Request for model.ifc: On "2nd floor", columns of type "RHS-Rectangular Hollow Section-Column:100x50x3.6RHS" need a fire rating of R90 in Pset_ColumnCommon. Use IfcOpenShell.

First a look at what the model holds.

```python
import ifcopenshell
import ifcopenshell.util.element

model = ifcopenshell.open("model.ifc")
print(model.schema)
storey = next(s for s in model.by_type("IfcBuildingStorey") if s.Name == "2nd floor")
columns = [e for e in ifcopenshell.util.element.get_decomposition(storey) if e.is_a("IfcColumn")]
seen = {}
for e in columns:
    element_type = ifcopenshell.util.element.get_type(e)
    key = (element_type.Name if element_type != e and element_type else None, ifcopenshell.util.element.get_pset(e, "Pset_ColumnCommon", "FireRating"))
    seen[key] = seen.get(key, 0) + 1
for (name, value), count in sorted(seen.items(), key=str):
    print(count, "x", name, "|", value)
```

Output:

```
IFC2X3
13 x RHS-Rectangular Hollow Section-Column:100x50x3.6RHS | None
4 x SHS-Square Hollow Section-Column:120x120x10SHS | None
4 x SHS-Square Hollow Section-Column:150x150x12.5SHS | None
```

```python
import ifcopenshell
import ifcopenshell.api.pset
import ifcopenshell.util.element

model = ifcopenshell.open("model.ifc")

storey = next(s for s in model.by_type("IfcBuildingStorey") if s.Name == "2nd floor")
columns = [e for e in ifcopenshell.util.element.get_decomposition(storey) if e.is_a("IfcColumn")]

count = 0
for e in columns:
    element_type = ifcopenshell.util.element.get_type(e)
    if element_type in (None, e) or element_type.Name != "RHS-Rectangular Hollow Section-Column:100x50x3.6RHS":
        continue
    # add_pset returns the element's existing set when there is one.
    pset = ifcopenshell.api.pset.add_pset(model, product=e, name="Pset_ColumnCommon")
    ifcopenshell.api.pset.edit_pset(model, pset=pset, properties={"FireRating": "R90"})
    count += 1

print(count, "columns updated")

model.write("model-out.ifc")
```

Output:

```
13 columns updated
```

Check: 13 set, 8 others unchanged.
